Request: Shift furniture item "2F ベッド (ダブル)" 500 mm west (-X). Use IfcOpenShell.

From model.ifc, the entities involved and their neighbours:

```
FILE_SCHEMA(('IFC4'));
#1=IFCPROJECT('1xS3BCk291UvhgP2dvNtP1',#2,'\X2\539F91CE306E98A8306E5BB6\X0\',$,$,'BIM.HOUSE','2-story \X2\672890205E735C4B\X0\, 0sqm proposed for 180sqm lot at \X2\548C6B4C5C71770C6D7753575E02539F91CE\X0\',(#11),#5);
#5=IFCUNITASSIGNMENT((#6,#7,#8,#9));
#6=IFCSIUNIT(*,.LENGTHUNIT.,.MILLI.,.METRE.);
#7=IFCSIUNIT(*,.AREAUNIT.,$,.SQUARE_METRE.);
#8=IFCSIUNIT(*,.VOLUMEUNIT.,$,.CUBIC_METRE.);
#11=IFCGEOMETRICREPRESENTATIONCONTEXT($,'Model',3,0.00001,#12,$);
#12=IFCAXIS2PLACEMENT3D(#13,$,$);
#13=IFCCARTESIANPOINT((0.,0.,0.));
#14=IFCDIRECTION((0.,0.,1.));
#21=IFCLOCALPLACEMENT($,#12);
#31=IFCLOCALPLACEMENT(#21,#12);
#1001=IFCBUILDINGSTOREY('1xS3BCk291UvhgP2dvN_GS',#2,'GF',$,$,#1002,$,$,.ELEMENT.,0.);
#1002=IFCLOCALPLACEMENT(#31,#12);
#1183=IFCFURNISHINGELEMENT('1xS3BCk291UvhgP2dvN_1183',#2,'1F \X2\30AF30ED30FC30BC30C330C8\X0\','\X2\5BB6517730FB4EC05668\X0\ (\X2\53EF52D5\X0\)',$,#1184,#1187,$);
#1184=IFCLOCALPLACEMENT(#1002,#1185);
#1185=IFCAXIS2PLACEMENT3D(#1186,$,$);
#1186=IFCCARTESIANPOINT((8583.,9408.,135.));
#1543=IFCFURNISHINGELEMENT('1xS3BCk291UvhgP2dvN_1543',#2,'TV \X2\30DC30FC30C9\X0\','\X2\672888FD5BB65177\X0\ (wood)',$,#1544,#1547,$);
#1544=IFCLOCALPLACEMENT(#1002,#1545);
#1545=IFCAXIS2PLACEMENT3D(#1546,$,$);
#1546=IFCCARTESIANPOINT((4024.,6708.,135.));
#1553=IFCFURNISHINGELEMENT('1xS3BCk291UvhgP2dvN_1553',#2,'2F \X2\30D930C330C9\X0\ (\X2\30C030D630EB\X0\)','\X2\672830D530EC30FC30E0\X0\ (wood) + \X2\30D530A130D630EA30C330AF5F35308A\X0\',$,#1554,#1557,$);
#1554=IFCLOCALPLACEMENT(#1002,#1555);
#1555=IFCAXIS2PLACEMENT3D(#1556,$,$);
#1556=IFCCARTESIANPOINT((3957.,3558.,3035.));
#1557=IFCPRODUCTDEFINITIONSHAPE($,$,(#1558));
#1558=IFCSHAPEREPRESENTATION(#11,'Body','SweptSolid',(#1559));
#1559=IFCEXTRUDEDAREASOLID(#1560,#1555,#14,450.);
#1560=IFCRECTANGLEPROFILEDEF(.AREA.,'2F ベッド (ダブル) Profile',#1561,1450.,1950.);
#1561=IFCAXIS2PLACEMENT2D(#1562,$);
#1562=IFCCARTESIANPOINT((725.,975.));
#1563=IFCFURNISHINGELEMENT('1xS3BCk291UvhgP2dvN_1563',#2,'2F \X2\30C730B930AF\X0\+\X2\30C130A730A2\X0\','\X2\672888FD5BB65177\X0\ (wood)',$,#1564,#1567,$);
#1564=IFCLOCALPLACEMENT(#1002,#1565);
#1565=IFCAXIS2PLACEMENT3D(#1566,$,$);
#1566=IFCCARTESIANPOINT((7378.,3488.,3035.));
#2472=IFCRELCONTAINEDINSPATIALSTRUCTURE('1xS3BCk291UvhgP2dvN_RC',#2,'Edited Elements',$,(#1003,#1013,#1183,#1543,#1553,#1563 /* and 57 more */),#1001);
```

```python
import ifcopenshell
import ifcopenshell.api.geometry
import ifcopenshell.util.placement
import ifcopenshell.util.unit

model = ifcopenshell.open("model.ifc")
unit_scale = ifcopenshell.util.unit.calculate_unit_scale(model)

item = model.by_guid("1xS3BCk291UvhgP2dvN_1553")
matrix = ifcopenshell.util.placement.get_local_placement(item.ObjectPlacement)
matrix[0, 3] -= 0.5 / unit_scale
ifcopenshell.api.geometry.edit_object_placement(model, product=item, matrix=matrix, is_si=False)

print(ifcopenshell.util.placement.get_local_placement(item.ObjectPlacement).round(3) + 0.0)

model.write("model_rev.ifc")
```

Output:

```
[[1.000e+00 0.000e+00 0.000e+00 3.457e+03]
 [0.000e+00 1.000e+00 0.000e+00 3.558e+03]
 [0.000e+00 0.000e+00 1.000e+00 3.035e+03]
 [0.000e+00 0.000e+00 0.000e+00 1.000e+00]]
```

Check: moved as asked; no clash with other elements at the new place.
